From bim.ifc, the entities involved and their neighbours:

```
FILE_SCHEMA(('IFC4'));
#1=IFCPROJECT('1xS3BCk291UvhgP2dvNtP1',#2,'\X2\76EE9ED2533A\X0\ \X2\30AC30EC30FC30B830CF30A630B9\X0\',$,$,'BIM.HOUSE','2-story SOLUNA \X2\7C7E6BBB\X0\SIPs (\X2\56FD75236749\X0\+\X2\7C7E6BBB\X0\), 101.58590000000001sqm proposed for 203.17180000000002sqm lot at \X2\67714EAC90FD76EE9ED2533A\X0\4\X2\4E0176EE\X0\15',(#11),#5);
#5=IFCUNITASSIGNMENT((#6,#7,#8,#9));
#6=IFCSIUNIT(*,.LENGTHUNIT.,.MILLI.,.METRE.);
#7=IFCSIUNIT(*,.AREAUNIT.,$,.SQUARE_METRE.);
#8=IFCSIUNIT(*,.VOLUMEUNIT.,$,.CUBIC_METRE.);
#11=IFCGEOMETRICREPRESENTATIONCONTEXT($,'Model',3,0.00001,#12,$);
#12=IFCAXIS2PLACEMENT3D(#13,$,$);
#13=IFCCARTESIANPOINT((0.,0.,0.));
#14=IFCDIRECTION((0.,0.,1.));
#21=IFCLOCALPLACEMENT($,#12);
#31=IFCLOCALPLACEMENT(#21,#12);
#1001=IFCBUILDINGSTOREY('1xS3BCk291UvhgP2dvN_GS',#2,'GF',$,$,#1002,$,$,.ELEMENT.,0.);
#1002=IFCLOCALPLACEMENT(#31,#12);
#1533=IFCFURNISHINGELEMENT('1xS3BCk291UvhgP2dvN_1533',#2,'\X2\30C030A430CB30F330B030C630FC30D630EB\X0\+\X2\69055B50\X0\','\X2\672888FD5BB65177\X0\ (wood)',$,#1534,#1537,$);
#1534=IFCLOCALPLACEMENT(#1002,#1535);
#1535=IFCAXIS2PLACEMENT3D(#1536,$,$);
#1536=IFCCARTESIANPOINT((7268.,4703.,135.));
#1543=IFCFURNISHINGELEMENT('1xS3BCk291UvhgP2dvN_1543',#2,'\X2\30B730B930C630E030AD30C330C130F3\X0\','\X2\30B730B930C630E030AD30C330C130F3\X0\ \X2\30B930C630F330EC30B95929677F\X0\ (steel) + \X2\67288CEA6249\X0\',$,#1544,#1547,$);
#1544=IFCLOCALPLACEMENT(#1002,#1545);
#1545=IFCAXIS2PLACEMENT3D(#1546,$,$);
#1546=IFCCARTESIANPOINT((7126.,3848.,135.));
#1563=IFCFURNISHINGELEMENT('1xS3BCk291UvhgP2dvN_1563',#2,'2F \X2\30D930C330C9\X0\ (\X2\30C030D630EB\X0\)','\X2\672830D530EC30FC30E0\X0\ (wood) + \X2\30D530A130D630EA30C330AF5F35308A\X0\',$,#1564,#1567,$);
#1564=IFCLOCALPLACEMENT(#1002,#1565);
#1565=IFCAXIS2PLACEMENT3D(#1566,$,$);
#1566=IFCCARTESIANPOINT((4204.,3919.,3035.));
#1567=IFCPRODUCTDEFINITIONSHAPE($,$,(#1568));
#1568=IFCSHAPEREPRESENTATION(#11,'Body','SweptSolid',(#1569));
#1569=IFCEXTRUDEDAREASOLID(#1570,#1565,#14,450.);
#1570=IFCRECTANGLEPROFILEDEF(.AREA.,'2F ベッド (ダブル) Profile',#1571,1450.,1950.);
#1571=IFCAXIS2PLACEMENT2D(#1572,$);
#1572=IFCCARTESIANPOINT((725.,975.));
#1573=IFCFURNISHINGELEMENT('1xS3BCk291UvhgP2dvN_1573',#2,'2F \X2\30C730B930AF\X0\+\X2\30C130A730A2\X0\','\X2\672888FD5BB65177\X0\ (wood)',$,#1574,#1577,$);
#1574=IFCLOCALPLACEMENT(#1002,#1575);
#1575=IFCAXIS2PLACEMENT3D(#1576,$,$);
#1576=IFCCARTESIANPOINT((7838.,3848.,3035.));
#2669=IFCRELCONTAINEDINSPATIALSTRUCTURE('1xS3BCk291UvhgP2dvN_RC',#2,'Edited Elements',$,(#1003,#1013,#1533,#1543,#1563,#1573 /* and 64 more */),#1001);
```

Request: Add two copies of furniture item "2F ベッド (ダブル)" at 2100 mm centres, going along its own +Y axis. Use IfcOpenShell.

```python
import ifcopenshell
import ifcopenshell.api.geometry
import ifcopenshell.api.root
import ifcopenshell.util.element
import ifcopenshell.util.placement

model = ifcopenshell.open("bim.ifc")


def reuse_history(source, copy):
    """copy_class also copies each property set's owner history, people and application; keep the originals."""
    for rel in copy.IsDefinedBy:
        if rel.is_a("IfcRelDefinesByProperties") and (history := rel.RelatingPropertyDefinition.OwnerHistory):
            rel.RelatingPropertyDefinition.OwnerHistory = source.OwnerHistory
            ifcopenshell.util.element.remove_deep2(model, history)


source = model.by_guid("1xS3BCk291UvhgP2dvN_1563")
base = ifcopenshell.util.placement.get_local_placement(source.ObjectPlacement)
step = base[:3, 1] * 2100.0

for i in range(1, 3):
    copy = ifcopenshell.api.root.copy_class(model, product=source)
    copy.Representation = ifcopenshell.util.element.copy_deep(
        model, source.Representation, exclude=["IfcGeometricRepresentationContext", "IfcRepresentationMap"]
    )
    reuse_history(source, copy)
    matrix = base.copy()
    matrix[:3, 3] += i * step
    print("added at", matrix[:3, 3].round(3) + 0.0)
    ifcopenshell.api.geometry.edit_object_placement(model, product=copy, matrix=matrix, is_si=False)

model.write("bim-out.ifc")
```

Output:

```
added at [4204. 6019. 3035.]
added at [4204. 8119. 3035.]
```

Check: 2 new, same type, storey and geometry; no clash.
